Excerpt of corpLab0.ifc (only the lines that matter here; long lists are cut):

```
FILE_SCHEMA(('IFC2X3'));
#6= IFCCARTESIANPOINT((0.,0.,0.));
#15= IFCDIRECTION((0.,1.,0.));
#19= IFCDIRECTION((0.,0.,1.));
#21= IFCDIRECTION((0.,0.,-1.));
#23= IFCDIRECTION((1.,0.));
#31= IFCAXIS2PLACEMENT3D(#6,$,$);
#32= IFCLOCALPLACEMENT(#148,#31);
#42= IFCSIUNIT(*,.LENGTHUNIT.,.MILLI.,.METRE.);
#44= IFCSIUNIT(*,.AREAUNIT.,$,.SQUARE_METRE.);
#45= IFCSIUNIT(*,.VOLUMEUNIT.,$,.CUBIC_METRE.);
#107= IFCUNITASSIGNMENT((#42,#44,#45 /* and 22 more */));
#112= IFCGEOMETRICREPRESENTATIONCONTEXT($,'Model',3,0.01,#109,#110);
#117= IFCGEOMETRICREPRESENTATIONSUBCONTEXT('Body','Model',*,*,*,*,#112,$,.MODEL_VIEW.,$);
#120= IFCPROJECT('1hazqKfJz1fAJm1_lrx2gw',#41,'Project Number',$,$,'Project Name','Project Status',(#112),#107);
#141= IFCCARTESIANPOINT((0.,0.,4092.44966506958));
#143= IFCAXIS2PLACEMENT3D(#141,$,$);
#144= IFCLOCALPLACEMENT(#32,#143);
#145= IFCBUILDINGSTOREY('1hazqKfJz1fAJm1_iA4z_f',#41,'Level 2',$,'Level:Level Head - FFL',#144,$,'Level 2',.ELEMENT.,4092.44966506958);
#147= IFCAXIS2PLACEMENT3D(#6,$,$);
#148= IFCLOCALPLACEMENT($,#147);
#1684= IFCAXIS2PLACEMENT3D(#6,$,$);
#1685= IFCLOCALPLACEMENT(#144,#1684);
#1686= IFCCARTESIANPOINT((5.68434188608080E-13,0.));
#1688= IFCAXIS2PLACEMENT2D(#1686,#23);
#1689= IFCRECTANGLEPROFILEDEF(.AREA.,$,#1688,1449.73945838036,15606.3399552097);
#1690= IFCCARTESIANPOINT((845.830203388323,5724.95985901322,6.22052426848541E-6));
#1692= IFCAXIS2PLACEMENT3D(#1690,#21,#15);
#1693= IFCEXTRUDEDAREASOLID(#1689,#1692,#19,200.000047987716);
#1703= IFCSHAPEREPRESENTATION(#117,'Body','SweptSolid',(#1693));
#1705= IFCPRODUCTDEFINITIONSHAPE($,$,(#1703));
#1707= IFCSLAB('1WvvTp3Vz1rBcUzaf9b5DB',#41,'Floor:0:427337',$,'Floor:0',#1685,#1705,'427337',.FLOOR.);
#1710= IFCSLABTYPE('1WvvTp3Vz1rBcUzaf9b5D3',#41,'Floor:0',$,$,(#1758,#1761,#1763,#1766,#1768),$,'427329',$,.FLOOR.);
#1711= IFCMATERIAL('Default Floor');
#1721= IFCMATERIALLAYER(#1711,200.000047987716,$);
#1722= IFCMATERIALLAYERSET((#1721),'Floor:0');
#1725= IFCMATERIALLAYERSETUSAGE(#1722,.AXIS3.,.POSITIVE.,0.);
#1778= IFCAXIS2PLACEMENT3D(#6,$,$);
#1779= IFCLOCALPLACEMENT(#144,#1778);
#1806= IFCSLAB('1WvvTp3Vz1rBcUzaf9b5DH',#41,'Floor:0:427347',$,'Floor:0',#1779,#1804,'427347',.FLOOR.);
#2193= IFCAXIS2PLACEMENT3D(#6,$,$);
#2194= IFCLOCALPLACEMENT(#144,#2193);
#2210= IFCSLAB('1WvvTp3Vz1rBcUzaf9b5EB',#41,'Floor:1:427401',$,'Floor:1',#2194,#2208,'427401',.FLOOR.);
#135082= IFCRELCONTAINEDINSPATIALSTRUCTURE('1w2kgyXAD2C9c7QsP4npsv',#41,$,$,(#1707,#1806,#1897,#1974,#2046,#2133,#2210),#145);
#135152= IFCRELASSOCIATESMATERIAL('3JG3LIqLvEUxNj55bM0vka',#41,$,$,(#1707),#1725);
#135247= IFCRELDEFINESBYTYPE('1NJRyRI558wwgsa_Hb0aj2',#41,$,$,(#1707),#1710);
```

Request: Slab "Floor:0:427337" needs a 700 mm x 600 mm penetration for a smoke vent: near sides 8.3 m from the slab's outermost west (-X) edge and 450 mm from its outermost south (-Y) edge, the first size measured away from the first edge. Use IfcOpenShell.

```python
import numpy as np
import ifcopenshell
import ifcopenshell.api.feature
import ifcopenshell.api.geometry
import ifcopenshell.api.root
import ifcopenshell.geom
import ifcopenshell.util.placement
import ifcopenshell.util.representation
import ifcopenshell.util.shape
import ifcopenshell.util.unit

model = ifcopenshell.open("corpLab0.ifc")
unit_scale = ifcopenshell.util.unit.calculate_unit_scale(model)
settings = ifcopenshell.geom.settings()


def volume(element):
    """Net volume in cubic metres, openings subtracted."""
    shape = ifcopenshell.geom.create_shape(settings, element)
    return ifcopenshell.util.shape.get_volume(shape.geometry)


slab = model.by_guid("1WvvTp3Vz1rBcUzaf9b5DB")
before = volume(slab)

# Extent in the slab's own axes, in metres. The edges named are its -X and -Y sides.
slab_shape = ifcopenshell.geom.create_shape(settings, slab)
vertices = ifcopenshell.util.shape.get_vertices(slab_shape.geometry)
x_min, y_min, bottom = vertices.min(axis=0)
top = vertices[:, 2].max()

opening = ifcopenshell.api.root.create_entity(model, ifc_class="IfcOpeningElement", name="Smoke vent opening")
context = ifcopenshell.util.representation.get_context(model, "Model", "Body", "MODEL_VIEW")
width, depth = 0.7, 0.6
outline = [(0.0, 0.0), (width, 0.0), (width, depth), (0.0, depth), (0.0, 0.0)]
# Overshoot both faces by 50 mm so the cut is clean.
shape = ifcopenshell.api.geometry.add_slab_representation(
    model, context=context, depth=top - bottom + 0.1, polyline=outline
)
ifcopenshell.api.geometry.assign_representation(model, product=opening, representation=shape)

matrix = ifcopenshell.util.placement.get_local_placement(slab.ObjectPlacement)
matrix[:, 3] = matrix @ np.append(np.array([x_min + 8.3, y_min + 0.45, bottom - 0.05]) / unit_scale, 1.0)
ifcopenshell.api.geometry.edit_object_placement(model, product=opening, matrix=matrix, is_si=False)
ifcopenshell.api.feature.add_feature(model, feature=opening, element=slab)

after = volume(slab)

print(f"slab volume {before:.3f} -> {after:.3f} m3")

model.write("corpLab0_edited.ifc")
```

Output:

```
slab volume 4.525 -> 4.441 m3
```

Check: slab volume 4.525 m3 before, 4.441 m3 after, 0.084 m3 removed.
